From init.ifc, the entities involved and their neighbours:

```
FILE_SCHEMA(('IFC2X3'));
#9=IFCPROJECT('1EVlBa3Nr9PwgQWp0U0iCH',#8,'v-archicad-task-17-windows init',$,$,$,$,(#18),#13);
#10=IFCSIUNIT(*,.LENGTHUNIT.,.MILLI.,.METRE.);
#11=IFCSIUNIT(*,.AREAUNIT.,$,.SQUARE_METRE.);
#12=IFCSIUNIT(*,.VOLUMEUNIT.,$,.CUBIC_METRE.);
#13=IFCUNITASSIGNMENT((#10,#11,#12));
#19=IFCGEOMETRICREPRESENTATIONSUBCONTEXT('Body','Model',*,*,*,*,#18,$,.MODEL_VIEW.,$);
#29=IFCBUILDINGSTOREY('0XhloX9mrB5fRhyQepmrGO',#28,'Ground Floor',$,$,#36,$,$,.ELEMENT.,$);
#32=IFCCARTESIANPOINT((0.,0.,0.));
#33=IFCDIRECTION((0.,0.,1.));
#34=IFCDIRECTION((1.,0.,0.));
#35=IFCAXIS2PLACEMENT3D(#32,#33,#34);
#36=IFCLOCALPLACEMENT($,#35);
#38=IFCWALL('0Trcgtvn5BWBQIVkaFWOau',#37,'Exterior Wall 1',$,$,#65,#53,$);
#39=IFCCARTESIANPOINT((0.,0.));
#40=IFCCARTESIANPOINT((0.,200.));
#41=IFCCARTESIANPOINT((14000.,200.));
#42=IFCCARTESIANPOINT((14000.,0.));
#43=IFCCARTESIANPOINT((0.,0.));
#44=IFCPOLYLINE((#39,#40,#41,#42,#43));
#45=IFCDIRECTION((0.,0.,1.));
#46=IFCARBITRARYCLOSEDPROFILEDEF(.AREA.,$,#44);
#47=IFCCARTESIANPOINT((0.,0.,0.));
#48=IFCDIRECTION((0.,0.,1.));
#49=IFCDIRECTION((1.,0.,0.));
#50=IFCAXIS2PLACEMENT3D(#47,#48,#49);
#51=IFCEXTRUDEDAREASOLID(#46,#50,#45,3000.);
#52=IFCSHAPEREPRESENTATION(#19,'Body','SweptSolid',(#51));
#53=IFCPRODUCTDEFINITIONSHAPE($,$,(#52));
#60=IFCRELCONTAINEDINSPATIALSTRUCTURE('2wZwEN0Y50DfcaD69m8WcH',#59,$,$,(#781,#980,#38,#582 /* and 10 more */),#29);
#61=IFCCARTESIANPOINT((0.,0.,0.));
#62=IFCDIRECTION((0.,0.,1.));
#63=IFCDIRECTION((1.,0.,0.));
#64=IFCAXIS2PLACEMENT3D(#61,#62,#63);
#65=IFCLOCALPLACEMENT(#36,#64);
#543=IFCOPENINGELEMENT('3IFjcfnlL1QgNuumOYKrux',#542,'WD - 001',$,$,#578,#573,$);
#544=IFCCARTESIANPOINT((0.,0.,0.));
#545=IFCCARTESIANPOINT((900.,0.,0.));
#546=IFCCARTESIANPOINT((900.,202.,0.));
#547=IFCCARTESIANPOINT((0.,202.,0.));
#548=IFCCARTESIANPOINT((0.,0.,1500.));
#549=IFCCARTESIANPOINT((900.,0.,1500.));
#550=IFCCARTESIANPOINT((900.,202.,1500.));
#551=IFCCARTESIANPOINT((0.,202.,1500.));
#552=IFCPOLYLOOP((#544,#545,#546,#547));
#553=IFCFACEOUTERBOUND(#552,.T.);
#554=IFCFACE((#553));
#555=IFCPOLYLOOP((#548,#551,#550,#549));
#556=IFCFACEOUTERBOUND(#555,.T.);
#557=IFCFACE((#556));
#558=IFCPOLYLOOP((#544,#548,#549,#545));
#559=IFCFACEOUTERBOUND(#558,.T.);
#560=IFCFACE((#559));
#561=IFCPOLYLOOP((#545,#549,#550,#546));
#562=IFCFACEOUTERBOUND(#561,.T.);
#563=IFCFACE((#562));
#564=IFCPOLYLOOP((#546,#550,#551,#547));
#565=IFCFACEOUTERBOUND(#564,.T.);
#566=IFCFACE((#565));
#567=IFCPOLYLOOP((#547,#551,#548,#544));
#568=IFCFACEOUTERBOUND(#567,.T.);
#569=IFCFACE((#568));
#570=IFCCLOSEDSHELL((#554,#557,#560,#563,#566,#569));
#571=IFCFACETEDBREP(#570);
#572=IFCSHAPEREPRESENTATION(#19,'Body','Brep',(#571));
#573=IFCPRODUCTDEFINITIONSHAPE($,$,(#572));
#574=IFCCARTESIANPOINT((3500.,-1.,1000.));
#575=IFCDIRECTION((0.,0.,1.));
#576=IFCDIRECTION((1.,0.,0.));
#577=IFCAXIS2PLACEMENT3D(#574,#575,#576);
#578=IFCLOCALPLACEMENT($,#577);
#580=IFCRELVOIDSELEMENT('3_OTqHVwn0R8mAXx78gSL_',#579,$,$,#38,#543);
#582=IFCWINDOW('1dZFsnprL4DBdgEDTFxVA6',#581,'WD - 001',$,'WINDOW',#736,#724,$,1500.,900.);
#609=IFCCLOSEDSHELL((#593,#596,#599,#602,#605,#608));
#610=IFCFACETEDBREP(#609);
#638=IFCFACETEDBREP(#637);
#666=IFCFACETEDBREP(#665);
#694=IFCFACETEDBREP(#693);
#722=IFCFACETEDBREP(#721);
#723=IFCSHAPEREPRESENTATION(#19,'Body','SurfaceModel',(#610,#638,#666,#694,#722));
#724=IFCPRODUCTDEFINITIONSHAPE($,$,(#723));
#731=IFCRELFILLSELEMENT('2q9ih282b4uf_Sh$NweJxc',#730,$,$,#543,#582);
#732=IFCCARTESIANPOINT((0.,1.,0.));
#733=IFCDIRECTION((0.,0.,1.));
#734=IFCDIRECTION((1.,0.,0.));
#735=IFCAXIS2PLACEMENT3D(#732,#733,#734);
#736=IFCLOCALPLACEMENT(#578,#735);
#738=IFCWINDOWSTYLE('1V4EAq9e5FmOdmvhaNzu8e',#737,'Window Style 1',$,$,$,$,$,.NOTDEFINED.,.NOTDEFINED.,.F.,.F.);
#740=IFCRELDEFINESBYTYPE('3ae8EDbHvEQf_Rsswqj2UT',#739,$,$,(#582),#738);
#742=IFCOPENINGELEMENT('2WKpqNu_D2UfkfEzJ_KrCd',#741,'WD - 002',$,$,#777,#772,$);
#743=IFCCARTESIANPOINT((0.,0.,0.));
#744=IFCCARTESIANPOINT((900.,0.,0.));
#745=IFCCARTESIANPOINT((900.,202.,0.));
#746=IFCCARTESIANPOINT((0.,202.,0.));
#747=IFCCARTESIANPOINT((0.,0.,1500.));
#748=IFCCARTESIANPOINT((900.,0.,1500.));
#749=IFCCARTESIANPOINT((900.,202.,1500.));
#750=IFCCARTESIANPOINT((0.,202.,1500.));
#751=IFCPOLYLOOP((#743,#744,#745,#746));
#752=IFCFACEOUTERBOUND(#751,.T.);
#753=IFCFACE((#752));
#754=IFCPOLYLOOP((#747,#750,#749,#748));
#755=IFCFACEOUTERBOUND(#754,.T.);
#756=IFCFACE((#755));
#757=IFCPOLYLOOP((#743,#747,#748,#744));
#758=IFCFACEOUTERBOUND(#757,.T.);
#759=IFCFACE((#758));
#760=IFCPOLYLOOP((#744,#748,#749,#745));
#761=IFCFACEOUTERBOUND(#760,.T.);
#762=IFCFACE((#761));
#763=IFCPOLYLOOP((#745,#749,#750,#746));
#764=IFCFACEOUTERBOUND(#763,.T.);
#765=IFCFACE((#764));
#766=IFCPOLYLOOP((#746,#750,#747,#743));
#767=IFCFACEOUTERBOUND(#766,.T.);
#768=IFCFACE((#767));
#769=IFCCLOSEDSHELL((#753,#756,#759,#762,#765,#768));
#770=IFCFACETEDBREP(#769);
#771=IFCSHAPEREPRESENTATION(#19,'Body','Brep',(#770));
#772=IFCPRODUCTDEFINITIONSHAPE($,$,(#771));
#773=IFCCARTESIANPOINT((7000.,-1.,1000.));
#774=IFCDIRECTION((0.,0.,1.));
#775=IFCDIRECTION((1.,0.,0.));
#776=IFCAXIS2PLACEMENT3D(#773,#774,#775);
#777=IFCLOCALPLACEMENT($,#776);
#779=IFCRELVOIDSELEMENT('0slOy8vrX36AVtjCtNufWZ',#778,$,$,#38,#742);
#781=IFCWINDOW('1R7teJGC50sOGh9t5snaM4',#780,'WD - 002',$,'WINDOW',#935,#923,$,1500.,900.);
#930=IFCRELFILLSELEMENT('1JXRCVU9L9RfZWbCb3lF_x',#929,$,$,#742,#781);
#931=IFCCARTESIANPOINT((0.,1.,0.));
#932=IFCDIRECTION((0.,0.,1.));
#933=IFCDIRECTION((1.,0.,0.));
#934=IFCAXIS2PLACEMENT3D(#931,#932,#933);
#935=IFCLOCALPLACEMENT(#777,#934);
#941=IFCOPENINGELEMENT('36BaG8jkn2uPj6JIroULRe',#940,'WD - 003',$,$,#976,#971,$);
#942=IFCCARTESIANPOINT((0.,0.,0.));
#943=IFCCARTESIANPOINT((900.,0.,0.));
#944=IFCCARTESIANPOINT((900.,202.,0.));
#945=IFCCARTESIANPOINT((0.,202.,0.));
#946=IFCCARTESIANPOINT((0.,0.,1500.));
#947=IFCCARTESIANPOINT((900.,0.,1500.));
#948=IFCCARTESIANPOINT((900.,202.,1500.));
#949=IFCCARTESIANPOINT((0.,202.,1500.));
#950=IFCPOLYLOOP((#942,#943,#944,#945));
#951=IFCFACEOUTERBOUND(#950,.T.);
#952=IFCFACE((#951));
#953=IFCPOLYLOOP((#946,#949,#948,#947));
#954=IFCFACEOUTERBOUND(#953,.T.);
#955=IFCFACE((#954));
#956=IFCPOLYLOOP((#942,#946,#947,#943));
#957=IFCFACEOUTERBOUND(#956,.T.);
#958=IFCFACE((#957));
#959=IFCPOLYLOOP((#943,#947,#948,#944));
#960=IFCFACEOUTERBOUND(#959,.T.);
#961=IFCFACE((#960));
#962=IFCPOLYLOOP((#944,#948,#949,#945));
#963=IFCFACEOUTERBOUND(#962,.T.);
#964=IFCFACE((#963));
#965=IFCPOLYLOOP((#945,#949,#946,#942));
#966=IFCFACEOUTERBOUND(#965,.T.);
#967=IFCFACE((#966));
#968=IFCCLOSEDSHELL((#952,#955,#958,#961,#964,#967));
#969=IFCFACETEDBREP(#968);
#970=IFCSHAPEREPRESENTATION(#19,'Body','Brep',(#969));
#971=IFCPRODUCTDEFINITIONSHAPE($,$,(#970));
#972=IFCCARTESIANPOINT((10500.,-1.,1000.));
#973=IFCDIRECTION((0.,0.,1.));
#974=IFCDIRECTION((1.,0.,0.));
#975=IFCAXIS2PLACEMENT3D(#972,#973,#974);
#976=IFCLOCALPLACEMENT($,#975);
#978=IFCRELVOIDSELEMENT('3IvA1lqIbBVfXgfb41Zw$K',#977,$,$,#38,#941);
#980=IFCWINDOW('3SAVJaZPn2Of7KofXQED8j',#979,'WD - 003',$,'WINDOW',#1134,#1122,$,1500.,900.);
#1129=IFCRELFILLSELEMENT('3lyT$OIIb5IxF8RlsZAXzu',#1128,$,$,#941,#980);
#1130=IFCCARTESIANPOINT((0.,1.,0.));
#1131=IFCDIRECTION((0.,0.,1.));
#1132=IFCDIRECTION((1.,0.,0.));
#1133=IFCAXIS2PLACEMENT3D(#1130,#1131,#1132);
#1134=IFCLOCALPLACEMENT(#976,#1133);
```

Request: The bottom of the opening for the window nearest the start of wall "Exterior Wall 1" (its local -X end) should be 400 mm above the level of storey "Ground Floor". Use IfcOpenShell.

```python
import numpy as np
import ifcopenshell
import ifcopenshell.api.geometry
import ifcopenshell.geom
import ifcopenshell.util.element
import ifcopenshell.util.placement
import ifcopenshell.util.shape
import ifcopenshell.util.unit

model = ifcopenshell.open("init.ifc")
unit_scale = ifcopenshell.util.unit.calculate_unit_scale(model)

window = model.by_guid("1dZFsnprL4DBdgEDTFxVA6")
opening = window.FillsVoids[0].RelatingOpeningElement
storey = ifcopenshell.util.element.get_container(window, ifc_class="IfcBuildingStorey")
level = ifcopenshell.util.placement.get_local_placement(storey.ObjectPlacement)[2, 3]

# The opening's origin need not be at the sill, so measure its lowest point.
shape = ifcopenshell.geom.create_shape(ifcopenshell.geom.settings(), opening)
bottom = ifcopenshell.util.shape.get_shape_bottom_elevation(shape, shape.geometry) / unit_scale
dz = level + 0.4 / unit_scale - bottom

shift = np.array([0.0, 0.0, dz])
# The window is placed relative to its opening, so it follows when the opening moves.
matrix = ifcopenshell.util.placement.get_local_placement(opening.ObjectPlacement)
matrix[:3, 3] += shift
ifcopenshell.api.geometry.edit_object_placement(
    model, product=opening, matrix=matrix, is_si=False, should_transform_children=True
)

print(f"moved by {dz * unit_scale:+.3f} m")

model.write("init-out.ifc")
```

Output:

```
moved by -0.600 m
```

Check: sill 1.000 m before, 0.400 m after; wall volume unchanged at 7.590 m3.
